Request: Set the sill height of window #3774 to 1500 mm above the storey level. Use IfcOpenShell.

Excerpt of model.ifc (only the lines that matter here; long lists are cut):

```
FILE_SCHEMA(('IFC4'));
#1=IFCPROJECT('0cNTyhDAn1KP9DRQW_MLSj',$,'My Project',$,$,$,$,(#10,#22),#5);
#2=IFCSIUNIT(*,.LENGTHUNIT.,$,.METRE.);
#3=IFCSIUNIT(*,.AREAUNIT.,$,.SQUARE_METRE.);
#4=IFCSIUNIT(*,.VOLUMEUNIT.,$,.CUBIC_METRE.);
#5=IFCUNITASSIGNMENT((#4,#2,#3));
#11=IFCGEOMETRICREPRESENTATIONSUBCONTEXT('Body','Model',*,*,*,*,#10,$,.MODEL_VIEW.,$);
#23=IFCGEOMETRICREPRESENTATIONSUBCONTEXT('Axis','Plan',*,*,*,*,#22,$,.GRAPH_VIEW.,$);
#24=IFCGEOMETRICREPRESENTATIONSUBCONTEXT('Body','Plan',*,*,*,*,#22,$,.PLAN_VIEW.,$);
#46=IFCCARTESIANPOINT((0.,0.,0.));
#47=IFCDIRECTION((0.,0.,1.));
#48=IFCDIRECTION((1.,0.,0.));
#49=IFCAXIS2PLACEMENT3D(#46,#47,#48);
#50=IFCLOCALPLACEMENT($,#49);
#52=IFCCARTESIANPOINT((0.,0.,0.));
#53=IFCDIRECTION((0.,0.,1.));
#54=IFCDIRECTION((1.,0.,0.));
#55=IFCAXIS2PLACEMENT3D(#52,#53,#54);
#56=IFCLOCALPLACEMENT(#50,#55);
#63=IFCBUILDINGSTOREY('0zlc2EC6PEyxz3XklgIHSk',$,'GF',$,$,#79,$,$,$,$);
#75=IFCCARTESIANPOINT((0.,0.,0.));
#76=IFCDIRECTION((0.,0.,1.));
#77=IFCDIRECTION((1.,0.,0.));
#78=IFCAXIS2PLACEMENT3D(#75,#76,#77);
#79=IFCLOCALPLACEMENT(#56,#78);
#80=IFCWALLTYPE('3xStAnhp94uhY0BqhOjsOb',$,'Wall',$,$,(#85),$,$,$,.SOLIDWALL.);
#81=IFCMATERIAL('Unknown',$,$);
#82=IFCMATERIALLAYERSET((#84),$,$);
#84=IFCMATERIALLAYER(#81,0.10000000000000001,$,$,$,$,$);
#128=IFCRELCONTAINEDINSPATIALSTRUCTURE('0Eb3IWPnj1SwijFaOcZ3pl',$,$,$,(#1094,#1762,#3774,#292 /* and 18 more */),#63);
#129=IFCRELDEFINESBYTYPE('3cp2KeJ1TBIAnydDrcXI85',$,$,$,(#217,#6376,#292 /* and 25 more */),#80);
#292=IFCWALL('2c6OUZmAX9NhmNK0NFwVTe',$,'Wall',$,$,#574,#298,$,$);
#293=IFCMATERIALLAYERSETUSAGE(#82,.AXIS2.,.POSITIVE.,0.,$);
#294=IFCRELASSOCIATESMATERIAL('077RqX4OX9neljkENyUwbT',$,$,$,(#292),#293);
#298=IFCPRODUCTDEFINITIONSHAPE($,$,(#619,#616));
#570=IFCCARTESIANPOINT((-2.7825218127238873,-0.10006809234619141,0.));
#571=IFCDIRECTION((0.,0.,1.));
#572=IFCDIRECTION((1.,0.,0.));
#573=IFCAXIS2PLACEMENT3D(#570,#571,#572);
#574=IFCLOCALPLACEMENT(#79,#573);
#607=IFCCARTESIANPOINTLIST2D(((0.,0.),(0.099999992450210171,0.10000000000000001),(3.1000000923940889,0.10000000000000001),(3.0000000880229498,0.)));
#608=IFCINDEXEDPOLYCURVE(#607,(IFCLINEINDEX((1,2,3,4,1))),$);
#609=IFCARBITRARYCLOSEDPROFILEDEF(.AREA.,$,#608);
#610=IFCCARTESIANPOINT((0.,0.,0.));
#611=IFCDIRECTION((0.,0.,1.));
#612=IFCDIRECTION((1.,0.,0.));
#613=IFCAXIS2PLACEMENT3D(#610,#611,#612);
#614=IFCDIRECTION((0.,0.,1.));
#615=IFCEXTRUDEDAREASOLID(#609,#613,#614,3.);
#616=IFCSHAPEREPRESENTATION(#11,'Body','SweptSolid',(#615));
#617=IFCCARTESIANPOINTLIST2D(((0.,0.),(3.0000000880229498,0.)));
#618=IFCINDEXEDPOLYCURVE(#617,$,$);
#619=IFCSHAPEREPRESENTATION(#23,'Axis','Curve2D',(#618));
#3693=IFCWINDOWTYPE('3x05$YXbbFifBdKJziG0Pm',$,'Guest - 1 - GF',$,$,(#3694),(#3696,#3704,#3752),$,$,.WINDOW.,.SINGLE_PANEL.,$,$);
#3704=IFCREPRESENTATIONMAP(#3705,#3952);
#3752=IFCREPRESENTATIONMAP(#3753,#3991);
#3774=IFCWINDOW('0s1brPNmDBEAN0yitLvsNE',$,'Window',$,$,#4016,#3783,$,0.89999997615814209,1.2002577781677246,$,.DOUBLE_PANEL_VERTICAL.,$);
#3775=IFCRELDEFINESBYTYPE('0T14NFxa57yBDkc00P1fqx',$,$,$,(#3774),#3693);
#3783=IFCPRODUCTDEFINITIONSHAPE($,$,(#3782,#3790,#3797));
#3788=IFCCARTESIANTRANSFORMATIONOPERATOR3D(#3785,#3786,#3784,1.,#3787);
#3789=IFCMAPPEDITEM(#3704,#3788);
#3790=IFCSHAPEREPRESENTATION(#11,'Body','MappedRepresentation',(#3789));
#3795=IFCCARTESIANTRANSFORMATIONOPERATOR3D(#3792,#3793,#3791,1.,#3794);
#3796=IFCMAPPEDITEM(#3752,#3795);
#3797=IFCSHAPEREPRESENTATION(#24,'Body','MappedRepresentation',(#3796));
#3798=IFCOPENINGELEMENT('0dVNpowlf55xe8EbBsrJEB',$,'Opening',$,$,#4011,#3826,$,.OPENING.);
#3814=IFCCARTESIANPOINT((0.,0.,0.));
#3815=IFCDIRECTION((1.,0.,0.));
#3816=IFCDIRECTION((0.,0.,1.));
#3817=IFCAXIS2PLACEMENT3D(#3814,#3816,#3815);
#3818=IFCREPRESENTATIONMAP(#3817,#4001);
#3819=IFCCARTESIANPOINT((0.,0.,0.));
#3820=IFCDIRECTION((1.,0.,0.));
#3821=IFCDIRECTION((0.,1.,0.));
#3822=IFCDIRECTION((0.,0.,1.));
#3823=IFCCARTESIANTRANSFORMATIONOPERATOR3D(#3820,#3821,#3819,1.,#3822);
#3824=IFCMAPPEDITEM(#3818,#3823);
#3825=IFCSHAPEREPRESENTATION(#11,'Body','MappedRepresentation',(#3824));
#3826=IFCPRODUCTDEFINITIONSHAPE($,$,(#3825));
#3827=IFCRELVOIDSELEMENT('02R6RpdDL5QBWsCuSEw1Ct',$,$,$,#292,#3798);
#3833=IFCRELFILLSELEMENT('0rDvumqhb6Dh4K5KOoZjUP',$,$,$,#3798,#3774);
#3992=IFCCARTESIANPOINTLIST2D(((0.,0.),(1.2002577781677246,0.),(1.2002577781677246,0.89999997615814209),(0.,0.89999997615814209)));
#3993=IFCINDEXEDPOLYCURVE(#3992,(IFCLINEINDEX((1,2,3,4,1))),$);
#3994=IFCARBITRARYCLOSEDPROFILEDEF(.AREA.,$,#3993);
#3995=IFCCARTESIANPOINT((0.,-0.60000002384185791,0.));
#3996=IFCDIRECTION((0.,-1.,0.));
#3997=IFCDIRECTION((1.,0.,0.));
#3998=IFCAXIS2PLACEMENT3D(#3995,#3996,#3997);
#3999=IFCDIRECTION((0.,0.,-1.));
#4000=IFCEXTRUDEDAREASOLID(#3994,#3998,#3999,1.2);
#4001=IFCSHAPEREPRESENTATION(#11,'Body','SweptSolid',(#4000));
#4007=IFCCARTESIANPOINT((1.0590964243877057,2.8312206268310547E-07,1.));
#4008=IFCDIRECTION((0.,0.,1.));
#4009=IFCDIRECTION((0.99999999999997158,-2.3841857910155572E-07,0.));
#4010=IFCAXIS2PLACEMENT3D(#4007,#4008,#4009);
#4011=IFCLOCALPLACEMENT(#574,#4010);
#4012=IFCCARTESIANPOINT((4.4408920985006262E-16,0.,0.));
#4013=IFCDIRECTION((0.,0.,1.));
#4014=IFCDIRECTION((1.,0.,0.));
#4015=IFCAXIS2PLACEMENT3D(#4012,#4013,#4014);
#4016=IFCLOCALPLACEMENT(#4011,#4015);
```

```python
import numpy as np
import ifcopenshell
import ifcopenshell.api.geometry
import ifcopenshell.geom
import ifcopenshell.util.element
import ifcopenshell.util.placement
import ifcopenshell.util.shape
import ifcopenshell.util.unit

model = ifcopenshell.open("model.ifc")
unit_scale = ifcopenshell.util.unit.calculate_unit_scale(model)

window = model.by_id(3774)
opening = window.FillsVoids[0].RelatingOpeningElement
storey = ifcopenshell.util.element.get_container(window, ifc_class="IfcBuildingStorey")
level = ifcopenshell.util.placement.get_local_placement(storey.ObjectPlacement)[2, 3]

# The opening's origin need not be at the sill, so measure its lowest point.
shape = ifcopenshell.geom.create_shape(ifcopenshell.geom.settings(), opening)
bottom = ifcopenshell.util.shape.get_shape_bottom_elevation(shape, shape.geometry) / unit_scale
dz = level + 1.5 / unit_scale - bottom

shift = np.array([0.0, 0.0, dz])
# The window is placed relative to its opening, so it follows when the opening moves.
matrix = ifcopenshell.util.placement.get_local_placement(opening.ObjectPlacement)
matrix[:3, 3] += shift
ifcopenshell.api.geometry.edit_object_placement(
    model, product=opening, matrix=matrix, is_si=False, should_transform_children=True
)

print(f"moved by {dz * unit_scale:+.3f} m")

model.write("model_edited.ifc")
```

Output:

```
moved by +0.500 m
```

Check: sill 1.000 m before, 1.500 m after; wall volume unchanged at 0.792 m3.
